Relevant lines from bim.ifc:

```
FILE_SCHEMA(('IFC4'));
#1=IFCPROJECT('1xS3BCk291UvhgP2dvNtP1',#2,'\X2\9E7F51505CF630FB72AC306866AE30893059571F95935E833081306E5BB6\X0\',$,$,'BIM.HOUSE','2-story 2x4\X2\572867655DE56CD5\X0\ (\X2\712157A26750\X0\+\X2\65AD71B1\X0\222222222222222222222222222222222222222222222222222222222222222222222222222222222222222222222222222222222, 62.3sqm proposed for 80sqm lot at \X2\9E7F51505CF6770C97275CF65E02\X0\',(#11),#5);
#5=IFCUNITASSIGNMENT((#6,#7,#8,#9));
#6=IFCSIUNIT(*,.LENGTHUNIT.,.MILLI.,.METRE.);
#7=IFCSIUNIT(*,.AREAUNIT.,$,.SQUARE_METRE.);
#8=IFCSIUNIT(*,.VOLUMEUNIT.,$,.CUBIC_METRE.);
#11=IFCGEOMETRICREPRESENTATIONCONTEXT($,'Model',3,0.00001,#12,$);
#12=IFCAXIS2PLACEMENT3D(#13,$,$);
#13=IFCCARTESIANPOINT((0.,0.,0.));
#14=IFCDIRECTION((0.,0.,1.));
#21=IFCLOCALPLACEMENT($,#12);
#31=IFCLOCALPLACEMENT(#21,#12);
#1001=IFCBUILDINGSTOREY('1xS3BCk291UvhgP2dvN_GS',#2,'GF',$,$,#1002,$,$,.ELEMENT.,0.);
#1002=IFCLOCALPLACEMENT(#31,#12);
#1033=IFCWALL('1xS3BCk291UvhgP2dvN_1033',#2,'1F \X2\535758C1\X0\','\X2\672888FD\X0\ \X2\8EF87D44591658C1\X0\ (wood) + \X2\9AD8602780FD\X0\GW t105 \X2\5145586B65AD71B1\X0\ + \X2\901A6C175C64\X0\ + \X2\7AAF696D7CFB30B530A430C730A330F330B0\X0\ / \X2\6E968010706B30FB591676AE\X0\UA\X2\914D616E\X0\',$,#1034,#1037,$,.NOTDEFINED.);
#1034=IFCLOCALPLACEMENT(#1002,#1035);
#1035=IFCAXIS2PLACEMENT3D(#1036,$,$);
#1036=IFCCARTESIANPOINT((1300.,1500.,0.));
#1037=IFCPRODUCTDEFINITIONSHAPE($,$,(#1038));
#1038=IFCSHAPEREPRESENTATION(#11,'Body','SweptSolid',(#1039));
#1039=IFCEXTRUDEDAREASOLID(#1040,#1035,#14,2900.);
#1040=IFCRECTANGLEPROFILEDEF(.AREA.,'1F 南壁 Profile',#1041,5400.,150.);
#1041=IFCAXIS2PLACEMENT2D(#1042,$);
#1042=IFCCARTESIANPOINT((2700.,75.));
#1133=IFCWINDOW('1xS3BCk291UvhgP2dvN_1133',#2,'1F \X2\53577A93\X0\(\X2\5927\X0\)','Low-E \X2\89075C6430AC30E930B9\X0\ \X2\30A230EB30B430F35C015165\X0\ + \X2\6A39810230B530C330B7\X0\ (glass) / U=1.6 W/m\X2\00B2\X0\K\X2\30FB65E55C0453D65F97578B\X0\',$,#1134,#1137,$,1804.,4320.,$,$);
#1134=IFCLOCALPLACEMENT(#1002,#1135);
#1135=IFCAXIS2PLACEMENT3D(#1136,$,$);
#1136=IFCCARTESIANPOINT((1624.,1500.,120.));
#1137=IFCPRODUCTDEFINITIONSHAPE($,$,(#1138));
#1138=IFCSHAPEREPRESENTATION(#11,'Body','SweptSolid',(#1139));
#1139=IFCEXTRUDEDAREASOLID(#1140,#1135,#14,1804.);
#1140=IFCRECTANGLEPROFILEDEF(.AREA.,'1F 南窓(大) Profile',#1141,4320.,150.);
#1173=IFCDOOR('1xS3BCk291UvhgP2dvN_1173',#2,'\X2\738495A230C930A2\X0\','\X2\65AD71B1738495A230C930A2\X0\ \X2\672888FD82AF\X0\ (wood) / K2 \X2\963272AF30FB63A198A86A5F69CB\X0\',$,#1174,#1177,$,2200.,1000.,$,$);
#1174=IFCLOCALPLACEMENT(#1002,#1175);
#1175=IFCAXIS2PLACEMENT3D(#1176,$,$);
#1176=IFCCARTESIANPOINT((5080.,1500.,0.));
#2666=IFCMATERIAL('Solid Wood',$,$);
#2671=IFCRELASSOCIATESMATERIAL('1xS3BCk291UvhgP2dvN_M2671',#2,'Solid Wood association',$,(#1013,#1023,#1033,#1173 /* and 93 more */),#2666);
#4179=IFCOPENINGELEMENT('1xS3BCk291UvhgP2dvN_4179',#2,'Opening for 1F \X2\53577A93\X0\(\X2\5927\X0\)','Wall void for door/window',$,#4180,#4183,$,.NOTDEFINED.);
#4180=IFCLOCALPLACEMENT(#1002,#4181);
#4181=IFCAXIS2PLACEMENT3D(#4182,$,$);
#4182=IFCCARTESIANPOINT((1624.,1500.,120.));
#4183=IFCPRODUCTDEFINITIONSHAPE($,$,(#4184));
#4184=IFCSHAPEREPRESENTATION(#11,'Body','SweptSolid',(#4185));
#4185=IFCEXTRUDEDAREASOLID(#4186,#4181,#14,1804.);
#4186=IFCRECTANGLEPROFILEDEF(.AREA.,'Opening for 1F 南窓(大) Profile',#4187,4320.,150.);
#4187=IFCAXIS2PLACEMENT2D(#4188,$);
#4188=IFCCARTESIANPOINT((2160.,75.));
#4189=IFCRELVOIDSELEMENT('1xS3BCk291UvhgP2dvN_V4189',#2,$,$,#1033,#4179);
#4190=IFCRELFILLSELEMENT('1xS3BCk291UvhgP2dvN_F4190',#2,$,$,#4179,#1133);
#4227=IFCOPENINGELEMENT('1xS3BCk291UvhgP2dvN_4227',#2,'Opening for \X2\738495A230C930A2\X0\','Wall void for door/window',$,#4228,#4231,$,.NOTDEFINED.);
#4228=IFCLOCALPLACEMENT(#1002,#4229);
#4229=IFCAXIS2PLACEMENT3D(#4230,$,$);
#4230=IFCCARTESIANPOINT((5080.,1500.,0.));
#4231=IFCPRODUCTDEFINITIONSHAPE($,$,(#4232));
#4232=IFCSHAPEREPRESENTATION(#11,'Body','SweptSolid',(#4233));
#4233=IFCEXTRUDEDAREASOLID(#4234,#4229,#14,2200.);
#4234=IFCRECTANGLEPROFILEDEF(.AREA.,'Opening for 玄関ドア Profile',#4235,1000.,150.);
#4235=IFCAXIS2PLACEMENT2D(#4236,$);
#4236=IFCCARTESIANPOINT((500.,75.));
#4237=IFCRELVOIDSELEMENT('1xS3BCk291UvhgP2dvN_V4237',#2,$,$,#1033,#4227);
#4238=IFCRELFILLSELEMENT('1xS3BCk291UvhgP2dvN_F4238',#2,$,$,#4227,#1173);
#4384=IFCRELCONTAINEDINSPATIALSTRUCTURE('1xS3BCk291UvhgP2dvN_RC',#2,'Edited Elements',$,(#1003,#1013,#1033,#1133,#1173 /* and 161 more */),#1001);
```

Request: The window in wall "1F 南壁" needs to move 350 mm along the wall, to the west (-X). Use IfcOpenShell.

```python
import ifcopenshell
import ifcopenshell.api.geometry
import ifcopenshell.util.placement
import ifcopenshell.util.unit

model = ifcopenshell.open("bim.ifc")
unit_scale = ifcopenshell.util.unit.calculate_unit_scale(model)

window = model.by_guid("1xS3BCk291UvhgP2dvN_1133")
opening = window.FillsVoids[0].RelatingOpeningElement
wall = opening.VoidsElements[0].RelatingBuildingElement

wall_matrix = ifcopenshell.util.placement.get_local_placement(wall.ObjectPlacement)
shift = wall_matrix[:3, 0] * -0.35 / unit_scale
before = ifcopenshell.util.placement.get_local_placement(window.ObjectPlacement)[:3, 3].copy()

# The window is not placed relative to its opening, so move both.
for product in (opening, window):
    matrix = ifcopenshell.util.placement.get_local_placement(product.ObjectPlacement)
    matrix[:3, 3] += shift
    ifcopenshell.api.geometry.edit_object_placement(model, product=product, matrix=matrix, is_si=False)

after = ifcopenshell.util.placement.get_local_placement(window.ObjectPlacement)[:3, 3]
print("window moved by", (after - before).round(3) + 0.0)

model.write("bim_rev.ifc")
```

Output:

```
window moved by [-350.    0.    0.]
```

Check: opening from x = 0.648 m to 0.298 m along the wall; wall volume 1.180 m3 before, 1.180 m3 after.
